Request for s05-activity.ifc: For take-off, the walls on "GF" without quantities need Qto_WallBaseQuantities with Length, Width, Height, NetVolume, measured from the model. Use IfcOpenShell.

First a look at what the model holds.

```python
import ifcopenshell
import ifcopenshell.util.element
import ifcopenshell.util.unit

model = ifcopenshell.open("s05-activity.ifc")
print(model.schema)
for unit_type in ("LENGTHUNIT", "AREAUNIT", "VOLUMEUNIT"):
    print(unit_type, ifcopenshell.util.unit.calculate_unit_scale(model, unit_type))
storey = next(s for s in model.by_type("IfcBuildingStorey") if s.Name == "GF")
walls = [e for e in ifcopenshell.util.element.get_decomposition(storey) if e.is_a("IfcWall")]
for e in sorted(walls, key=lambda e: e.id()):
    print(e.id(), e.is_a(), e.Name, list(ifcopenshell.util.element.get_psets(e, qtos_only=True)), sep=" | ")
```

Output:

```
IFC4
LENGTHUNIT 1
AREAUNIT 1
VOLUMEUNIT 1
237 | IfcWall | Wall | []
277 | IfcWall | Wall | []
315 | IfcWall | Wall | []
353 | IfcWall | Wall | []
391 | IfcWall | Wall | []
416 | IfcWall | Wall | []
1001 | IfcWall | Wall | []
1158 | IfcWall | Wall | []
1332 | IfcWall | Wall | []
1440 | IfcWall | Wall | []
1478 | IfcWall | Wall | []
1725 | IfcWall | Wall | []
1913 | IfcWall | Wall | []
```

```python
import ifcopenshell
import ifcopenshell.api.pset
import ifcopenshell.geom
import ifcopenshell.util.element
import ifcopenshell.util.shape
import ifcopenshell.util.unit

model = ifcopenshell.open("s05-activity.ifc")
unit_scale = ifcopenshell.util.unit.calculate_unit_scale(model)
volume_scale = ifcopenshell.util.unit.calculate_unit_scale(model, "VOLUMEUNIT")
settings = ifcopenshell.geom.settings()

storey = next(s for s in model.by_type("IfcBuildingStorey") if s.Name == "GF")
walls = [e for e in ifcopenshell.util.element.get_decomposition(storey) if e.is_a("IfcWall")]

for e in sorted(walls, key=lambda e: e.id()):
    if ifcopenshell.util.element.get_psets(e, qtos_only=True, should_inherit=False):
        continue
    # Geometry comes back in metres, in the element's own axes.
    shape = ifcopenshell.geom.create_shape(settings, e)
    values = {
        "Length": ifcopenshell.util.shape.get_x(shape.geometry) / unit_scale,
        "Width": ifcopenshell.util.shape.get_y(shape.geometry) / unit_scale,
        "Height": ifcopenshell.util.shape.get_z(shape.geometry) / unit_scale,
        "NetVolume": ifcopenshell.util.shape.get_volume(shape.geometry) / volume_scale,
    }
    qto = ifcopenshell.api.pset.add_qto(model, product=e, name="Qto_WallBaseQuantities")
    ifcopenshell.api.pset.edit_qto(model, qto=qto, properties=values)
    print(e.id(), {k: round(v, 3) for k, v in values.items()})

model.write("s05-activity_edited.ifc")
```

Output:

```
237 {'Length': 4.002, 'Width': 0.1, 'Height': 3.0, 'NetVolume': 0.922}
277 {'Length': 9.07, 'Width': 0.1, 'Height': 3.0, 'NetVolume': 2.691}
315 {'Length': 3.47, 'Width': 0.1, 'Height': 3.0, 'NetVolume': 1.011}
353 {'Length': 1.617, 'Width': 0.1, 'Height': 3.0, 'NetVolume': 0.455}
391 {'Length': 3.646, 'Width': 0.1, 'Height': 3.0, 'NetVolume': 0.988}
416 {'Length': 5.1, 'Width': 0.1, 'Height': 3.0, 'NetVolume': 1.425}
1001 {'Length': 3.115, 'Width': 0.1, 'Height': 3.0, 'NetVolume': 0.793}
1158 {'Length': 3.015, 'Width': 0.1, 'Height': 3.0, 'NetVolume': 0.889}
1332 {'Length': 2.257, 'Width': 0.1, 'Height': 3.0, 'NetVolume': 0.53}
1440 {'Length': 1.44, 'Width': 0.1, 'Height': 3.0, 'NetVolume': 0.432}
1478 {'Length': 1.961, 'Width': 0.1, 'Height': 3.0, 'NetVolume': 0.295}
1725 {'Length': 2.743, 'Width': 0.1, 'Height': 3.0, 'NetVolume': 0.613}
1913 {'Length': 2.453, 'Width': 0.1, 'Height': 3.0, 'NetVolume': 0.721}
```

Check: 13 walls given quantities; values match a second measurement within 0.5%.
